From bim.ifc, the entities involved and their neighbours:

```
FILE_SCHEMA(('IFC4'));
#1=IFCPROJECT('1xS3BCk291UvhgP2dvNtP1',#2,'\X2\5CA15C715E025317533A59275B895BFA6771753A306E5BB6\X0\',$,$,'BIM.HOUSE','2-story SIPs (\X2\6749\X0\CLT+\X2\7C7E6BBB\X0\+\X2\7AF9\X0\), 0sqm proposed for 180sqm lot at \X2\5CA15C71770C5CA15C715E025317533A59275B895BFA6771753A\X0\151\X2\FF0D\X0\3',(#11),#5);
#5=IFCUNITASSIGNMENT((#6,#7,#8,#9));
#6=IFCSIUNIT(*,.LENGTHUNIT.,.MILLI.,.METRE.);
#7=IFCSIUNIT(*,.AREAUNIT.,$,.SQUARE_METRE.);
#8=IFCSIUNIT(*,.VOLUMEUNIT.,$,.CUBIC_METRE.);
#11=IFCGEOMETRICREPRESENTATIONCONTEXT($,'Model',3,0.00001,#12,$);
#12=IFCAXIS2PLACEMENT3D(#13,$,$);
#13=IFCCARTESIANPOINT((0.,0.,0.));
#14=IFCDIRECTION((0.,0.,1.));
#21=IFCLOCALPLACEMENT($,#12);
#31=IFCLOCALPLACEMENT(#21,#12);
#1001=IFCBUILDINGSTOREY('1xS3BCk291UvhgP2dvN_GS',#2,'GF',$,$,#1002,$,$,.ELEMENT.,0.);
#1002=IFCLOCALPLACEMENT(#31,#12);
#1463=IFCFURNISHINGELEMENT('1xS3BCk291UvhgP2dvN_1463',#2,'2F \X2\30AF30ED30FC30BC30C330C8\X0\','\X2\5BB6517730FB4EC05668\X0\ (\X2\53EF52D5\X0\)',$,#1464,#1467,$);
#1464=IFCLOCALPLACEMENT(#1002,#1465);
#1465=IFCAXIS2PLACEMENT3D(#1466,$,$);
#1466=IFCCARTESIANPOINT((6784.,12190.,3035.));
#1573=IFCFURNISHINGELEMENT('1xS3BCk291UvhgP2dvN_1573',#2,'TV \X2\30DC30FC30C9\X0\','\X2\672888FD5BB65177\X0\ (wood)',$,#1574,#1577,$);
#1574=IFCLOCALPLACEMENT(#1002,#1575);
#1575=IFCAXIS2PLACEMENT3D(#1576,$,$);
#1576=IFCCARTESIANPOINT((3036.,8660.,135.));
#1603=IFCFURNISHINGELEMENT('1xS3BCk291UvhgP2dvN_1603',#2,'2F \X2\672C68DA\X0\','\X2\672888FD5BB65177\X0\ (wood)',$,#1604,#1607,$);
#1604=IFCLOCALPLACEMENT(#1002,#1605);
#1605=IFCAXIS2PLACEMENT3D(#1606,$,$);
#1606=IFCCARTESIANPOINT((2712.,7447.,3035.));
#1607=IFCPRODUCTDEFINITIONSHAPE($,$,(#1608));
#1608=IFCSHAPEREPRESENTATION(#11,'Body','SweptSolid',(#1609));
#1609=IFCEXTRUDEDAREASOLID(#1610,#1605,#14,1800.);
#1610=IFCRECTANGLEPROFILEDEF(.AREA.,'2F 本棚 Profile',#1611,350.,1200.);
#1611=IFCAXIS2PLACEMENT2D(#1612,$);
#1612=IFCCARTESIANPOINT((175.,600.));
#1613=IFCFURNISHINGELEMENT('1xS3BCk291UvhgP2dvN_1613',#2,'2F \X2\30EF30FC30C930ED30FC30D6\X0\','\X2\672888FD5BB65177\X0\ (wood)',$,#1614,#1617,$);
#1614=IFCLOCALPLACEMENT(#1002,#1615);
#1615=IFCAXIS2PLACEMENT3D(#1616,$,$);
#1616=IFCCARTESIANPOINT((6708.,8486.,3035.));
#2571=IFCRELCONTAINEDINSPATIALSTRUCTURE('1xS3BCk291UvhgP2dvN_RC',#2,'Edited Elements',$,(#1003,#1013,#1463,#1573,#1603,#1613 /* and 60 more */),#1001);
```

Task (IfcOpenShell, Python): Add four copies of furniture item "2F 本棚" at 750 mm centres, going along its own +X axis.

```python
import ifcopenshell
import ifcopenshell.api.geometry
import ifcopenshell.api.root
import ifcopenshell.util.element
import ifcopenshell.util.placement
import ifcopenshell.util.unit

model = ifcopenshell.open("bim.ifc")
unit_scale = ifcopenshell.util.unit.calculate_unit_scale(model)


def reuse_history(source, copy):
    """copy_class also copies each property set's owner history, people and application; keep the originals."""
    for rel in copy.IsDefinedBy:
        if rel.is_a("IfcRelDefinesByProperties") and (history := rel.RelatingPropertyDefinition.OwnerHistory):
            rel.RelatingPropertyDefinition.OwnerHistory = source.OwnerHistory
            ifcopenshell.util.element.remove_deep2(model, history)


source = model.by_id(1603)
base = ifcopenshell.util.placement.get_local_placement(source.ObjectPlacement)
step = base[:3, 0] * 0.75 / unit_scale

for i in range(1, 5):
    copy = ifcopenshell.api.root.copy_class(model, product=source)
    copy.Representation = ifcopenshell.util.element.copy_deep(
        model, source.Representation, exclude=["IfcGeometricRepresentationContext", "IfcRepresentationMap"]
    )
    reuse_history(source, copy)
    matrix = base.copy()
    matrix[:3, 3] += i * step
    print("added at", matrix[:3, 3].round(3) + 0.0)
    ifcopenshell.api.geometry.edit_object_placement(model, product=copy, matrix=matrix, is_si=False)

model.write("bim-out.ifc")
```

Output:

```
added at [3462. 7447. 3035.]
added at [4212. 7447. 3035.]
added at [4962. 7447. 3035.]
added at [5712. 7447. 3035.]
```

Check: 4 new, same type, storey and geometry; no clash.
